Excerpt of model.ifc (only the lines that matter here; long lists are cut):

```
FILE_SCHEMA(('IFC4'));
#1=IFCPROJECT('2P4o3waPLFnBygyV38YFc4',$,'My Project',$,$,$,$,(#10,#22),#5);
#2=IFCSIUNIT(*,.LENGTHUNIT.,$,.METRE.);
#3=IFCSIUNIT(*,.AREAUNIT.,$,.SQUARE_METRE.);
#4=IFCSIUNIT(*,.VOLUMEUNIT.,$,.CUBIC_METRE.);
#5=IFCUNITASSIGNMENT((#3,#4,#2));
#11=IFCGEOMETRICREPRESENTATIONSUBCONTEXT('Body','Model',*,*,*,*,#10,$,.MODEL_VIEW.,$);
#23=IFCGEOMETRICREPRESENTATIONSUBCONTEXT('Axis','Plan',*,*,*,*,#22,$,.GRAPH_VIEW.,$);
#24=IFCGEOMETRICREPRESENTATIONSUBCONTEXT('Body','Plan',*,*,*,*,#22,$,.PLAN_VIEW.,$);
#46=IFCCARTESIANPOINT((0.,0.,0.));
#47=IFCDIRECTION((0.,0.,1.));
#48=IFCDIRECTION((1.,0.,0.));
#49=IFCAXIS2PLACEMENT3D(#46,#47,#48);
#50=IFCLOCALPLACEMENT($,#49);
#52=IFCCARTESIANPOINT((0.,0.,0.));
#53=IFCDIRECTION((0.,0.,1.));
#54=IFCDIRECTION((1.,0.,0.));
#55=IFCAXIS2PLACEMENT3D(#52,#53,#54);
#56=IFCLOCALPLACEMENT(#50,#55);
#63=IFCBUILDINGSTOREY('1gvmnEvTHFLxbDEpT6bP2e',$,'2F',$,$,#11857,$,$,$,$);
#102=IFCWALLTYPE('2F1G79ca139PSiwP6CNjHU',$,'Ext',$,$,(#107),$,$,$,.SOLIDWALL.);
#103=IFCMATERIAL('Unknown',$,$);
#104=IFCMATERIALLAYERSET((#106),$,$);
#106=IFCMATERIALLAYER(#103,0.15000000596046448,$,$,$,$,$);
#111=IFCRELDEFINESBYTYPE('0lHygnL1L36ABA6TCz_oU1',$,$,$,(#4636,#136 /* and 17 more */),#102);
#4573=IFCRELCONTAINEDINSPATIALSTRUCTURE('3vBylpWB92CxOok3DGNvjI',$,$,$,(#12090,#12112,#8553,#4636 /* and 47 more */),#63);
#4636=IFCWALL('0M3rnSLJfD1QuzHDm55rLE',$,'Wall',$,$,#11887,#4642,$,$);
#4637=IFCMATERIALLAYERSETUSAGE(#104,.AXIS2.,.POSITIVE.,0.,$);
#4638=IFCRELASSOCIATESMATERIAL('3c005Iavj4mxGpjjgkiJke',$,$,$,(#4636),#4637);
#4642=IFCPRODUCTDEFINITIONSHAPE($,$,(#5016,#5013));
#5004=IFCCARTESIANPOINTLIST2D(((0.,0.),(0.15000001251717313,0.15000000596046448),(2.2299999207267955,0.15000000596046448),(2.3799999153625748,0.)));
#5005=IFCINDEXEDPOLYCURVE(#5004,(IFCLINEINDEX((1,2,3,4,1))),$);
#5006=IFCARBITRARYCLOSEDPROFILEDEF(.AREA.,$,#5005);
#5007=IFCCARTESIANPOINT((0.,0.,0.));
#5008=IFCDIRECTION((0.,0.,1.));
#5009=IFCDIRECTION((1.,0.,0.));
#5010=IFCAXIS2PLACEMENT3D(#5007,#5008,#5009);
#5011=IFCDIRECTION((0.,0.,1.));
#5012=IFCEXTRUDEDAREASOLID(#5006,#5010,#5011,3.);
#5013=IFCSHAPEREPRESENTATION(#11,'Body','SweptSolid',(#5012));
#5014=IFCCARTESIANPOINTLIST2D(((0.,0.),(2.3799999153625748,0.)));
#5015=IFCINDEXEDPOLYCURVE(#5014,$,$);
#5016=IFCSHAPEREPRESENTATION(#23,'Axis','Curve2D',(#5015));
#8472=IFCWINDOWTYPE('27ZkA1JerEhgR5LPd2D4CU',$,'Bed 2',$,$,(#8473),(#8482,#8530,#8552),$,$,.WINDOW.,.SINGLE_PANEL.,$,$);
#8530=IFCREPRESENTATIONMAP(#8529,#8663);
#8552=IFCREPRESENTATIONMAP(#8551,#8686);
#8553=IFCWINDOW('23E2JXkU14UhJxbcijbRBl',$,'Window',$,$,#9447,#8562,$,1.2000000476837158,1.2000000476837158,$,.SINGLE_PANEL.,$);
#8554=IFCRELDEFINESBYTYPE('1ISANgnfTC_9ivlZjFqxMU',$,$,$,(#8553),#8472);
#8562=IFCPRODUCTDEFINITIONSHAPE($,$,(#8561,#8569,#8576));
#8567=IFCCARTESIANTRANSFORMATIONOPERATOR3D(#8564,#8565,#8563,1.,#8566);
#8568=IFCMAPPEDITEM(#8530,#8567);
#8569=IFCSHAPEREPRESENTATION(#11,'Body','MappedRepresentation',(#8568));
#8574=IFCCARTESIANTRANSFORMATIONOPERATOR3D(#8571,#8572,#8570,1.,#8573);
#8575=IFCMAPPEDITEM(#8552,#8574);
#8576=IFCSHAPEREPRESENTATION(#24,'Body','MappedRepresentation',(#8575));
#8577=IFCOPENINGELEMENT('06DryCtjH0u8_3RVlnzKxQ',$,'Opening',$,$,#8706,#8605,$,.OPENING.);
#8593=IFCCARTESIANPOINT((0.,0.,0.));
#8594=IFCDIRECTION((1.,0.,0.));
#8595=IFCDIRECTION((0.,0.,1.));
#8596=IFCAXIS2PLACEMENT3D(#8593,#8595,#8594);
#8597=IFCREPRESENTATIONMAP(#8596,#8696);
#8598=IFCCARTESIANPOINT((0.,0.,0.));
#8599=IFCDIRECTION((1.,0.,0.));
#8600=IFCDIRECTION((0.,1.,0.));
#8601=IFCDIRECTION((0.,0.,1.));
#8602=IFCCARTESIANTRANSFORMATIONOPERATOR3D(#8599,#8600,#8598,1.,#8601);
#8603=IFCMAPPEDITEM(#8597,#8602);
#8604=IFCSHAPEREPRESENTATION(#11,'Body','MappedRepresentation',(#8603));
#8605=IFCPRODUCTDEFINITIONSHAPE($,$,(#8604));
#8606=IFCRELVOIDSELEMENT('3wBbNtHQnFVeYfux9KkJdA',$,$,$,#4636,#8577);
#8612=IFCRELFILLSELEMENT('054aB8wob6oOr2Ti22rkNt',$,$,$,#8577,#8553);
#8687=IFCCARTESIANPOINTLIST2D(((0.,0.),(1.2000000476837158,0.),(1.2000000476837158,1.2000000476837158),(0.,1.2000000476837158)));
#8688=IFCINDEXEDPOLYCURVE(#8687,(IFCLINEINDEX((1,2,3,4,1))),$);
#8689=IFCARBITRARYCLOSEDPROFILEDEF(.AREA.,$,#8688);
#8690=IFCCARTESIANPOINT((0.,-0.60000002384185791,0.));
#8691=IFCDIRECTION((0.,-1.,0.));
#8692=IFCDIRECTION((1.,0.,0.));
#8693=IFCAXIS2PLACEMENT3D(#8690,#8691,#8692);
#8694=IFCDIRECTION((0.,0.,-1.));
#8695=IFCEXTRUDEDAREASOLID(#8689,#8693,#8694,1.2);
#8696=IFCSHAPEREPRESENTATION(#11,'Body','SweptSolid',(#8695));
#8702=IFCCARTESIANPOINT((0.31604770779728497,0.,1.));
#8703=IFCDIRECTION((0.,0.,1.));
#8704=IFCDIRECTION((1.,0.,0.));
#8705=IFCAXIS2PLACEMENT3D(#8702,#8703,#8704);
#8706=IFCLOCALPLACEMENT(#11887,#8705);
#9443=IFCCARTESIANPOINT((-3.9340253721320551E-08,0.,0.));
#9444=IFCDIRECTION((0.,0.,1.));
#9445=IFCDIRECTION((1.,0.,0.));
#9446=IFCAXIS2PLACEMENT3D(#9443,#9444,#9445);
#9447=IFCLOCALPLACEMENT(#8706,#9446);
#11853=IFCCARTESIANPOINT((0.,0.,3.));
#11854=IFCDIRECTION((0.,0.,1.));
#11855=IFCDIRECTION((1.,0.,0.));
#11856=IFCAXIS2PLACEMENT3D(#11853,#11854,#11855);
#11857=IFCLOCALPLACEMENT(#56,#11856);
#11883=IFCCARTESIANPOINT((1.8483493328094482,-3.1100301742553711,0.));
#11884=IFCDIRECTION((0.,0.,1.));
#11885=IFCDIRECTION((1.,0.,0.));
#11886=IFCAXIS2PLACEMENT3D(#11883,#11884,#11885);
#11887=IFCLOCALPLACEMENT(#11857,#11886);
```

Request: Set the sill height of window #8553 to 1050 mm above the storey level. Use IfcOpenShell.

```python
import numpy as np
import ifcopenshell
import ifcopenshell.api.geometry
import ifcopenshell.geom
import ifcopenshell.util.element
import ifcopenshell.util.placement
import ifcopenshell.util.shape
import ifcopenshell.util.unit

model = ifcopenshell.open("model.ifc")
unit_scale = ifcopenshell.util.unit.calculate_unit_scale(model)

window = model.by_id(8553)
opening = window.FillsVoids[0].RelatingOpeningElement
storey = ifcopenshell.util.element.get_container(window, ifc_class="IfcBuildingStorey")
level = ifcopenshell.util.placement.get_local_placement(storey.ObjectPlacement)[2, 3]

# The opening's origin need not be at the sill, so measure its lowest point.
shape = ifcopenshell.geom.create_shape(ifcopenshell.geom.settings(), opening)
bottom = ifcopenshell.util.shape.get_shape_bottom_elevation(shape, shape.geometry) / unit_scale
dz = level + 1.05 / unit_scale - bottom

shift = np.array([0.0, 0.0, dz])
# The window is placed relative to its opening, so it follows when the opening moves.
matrix = ifcopenshell.util.placement.get_local_placement(opening.ObjectPlacement)
matrix[:3, 3] += shift
ifcopenshell.api.geometry.edit_object_placement(
    model, product=opening, matrix=matrix, is_si=False, should_transform_children=True
)

print(f"moved by {dz * unit_scale:+.3f} m")

model.write("model_rev.ifc")
```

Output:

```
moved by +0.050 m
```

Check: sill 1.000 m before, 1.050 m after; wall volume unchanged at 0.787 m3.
